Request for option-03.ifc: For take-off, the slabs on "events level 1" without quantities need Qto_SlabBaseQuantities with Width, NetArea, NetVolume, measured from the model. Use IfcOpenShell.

First a look at what the model holds.

```python
import ifcopenshell
import ifcopenshell.util.element
import ifcopenshell.util.unit

model = ifcopenshell.open("option-03.ifc")
print(model.schema)
for unit_type in ("LENGTHUNIT", "AREAUNIT", "VOLUMEUNIT"):
    print(unit_type, ifcopenshell.util.unit.calculate_unit_scale(model, unit_type))
storey = next(s for s in model.by_type("IfcBuildingStorey") if s.Name == "events level 1")
slabs = [e for e in ifcopenshell.util.element.get_decomposition(storey) if e.is_a("IfcSlab")]
for e in sorted(slabs, key=lambda e: e.id()):
    print(e.id(), e.is_a(), e.Name, list(ifcopenshell.util.element.get_psets(e, qtos_only=True)), sep=" | ")
```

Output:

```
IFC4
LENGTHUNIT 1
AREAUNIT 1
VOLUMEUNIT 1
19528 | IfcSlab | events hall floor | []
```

```python
import ifcopenshell
import ifcopenshell.api.pset
import ifcopenshell.geom
import ifcopenshell.util.element
import ifcopenshell.util.shape
import ifcopenshell.util.unit

model = ifcopenshell.open("option-03.ifc")
unit_scale = ifcopenshell.util.unit.calculate_unit_scale(model)
area_scale = ifcopenshell.util.unit.calculate_unit_scale(model, "AREAUNIT")
volume_scale = ifcopenshell.util.unit.calculate_unit_scale(model, "VOLUMEUNIT")
settings = ifcopenshell.geom.settings()

storey = next(s for s in model.by_type("IfcBuildingStorey") if s.Name == "events level 1")
slabs = [e for e in ifcopenshell.util.element.get_decomposition(storey) if e.is_a("IfcSlab")]

for e in sorted(slabs, key=lambda e: e.id()):
    if ifcopenshell.util.element.get_psets(e, qtos_only=True, should_inherit=False):
        continue
    # Geometry comes back in metres, in the element's own axes.
    shape = ifcopenshell.geom.create_shape(settings, e)
    values = {
        "Width": ifcopenshell.util.shape.get_z(shape.geometry) / unit_scale,
        "NetArea": ifcopenshell.util.shape.get_footprint_area(shape.geometry) / area_scale,
        "NetVolume": ifcopenshell.util.shape.get_volume(shape.geometry) / volume_scale,
    }
    qto = ifcopenshell.api.pset.add_qto(model, product=e, name="Qto_SlabBaseQuantities")
    ifcopenshell.api.pset.edit_qto(model, qto=qto, properties=values)
    print(e.id(), {k: round(v, 3) for k, v in values.items()})

model.write("option-03_updated.ifc")
```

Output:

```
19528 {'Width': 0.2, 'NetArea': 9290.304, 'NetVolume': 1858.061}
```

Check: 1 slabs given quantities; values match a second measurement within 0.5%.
